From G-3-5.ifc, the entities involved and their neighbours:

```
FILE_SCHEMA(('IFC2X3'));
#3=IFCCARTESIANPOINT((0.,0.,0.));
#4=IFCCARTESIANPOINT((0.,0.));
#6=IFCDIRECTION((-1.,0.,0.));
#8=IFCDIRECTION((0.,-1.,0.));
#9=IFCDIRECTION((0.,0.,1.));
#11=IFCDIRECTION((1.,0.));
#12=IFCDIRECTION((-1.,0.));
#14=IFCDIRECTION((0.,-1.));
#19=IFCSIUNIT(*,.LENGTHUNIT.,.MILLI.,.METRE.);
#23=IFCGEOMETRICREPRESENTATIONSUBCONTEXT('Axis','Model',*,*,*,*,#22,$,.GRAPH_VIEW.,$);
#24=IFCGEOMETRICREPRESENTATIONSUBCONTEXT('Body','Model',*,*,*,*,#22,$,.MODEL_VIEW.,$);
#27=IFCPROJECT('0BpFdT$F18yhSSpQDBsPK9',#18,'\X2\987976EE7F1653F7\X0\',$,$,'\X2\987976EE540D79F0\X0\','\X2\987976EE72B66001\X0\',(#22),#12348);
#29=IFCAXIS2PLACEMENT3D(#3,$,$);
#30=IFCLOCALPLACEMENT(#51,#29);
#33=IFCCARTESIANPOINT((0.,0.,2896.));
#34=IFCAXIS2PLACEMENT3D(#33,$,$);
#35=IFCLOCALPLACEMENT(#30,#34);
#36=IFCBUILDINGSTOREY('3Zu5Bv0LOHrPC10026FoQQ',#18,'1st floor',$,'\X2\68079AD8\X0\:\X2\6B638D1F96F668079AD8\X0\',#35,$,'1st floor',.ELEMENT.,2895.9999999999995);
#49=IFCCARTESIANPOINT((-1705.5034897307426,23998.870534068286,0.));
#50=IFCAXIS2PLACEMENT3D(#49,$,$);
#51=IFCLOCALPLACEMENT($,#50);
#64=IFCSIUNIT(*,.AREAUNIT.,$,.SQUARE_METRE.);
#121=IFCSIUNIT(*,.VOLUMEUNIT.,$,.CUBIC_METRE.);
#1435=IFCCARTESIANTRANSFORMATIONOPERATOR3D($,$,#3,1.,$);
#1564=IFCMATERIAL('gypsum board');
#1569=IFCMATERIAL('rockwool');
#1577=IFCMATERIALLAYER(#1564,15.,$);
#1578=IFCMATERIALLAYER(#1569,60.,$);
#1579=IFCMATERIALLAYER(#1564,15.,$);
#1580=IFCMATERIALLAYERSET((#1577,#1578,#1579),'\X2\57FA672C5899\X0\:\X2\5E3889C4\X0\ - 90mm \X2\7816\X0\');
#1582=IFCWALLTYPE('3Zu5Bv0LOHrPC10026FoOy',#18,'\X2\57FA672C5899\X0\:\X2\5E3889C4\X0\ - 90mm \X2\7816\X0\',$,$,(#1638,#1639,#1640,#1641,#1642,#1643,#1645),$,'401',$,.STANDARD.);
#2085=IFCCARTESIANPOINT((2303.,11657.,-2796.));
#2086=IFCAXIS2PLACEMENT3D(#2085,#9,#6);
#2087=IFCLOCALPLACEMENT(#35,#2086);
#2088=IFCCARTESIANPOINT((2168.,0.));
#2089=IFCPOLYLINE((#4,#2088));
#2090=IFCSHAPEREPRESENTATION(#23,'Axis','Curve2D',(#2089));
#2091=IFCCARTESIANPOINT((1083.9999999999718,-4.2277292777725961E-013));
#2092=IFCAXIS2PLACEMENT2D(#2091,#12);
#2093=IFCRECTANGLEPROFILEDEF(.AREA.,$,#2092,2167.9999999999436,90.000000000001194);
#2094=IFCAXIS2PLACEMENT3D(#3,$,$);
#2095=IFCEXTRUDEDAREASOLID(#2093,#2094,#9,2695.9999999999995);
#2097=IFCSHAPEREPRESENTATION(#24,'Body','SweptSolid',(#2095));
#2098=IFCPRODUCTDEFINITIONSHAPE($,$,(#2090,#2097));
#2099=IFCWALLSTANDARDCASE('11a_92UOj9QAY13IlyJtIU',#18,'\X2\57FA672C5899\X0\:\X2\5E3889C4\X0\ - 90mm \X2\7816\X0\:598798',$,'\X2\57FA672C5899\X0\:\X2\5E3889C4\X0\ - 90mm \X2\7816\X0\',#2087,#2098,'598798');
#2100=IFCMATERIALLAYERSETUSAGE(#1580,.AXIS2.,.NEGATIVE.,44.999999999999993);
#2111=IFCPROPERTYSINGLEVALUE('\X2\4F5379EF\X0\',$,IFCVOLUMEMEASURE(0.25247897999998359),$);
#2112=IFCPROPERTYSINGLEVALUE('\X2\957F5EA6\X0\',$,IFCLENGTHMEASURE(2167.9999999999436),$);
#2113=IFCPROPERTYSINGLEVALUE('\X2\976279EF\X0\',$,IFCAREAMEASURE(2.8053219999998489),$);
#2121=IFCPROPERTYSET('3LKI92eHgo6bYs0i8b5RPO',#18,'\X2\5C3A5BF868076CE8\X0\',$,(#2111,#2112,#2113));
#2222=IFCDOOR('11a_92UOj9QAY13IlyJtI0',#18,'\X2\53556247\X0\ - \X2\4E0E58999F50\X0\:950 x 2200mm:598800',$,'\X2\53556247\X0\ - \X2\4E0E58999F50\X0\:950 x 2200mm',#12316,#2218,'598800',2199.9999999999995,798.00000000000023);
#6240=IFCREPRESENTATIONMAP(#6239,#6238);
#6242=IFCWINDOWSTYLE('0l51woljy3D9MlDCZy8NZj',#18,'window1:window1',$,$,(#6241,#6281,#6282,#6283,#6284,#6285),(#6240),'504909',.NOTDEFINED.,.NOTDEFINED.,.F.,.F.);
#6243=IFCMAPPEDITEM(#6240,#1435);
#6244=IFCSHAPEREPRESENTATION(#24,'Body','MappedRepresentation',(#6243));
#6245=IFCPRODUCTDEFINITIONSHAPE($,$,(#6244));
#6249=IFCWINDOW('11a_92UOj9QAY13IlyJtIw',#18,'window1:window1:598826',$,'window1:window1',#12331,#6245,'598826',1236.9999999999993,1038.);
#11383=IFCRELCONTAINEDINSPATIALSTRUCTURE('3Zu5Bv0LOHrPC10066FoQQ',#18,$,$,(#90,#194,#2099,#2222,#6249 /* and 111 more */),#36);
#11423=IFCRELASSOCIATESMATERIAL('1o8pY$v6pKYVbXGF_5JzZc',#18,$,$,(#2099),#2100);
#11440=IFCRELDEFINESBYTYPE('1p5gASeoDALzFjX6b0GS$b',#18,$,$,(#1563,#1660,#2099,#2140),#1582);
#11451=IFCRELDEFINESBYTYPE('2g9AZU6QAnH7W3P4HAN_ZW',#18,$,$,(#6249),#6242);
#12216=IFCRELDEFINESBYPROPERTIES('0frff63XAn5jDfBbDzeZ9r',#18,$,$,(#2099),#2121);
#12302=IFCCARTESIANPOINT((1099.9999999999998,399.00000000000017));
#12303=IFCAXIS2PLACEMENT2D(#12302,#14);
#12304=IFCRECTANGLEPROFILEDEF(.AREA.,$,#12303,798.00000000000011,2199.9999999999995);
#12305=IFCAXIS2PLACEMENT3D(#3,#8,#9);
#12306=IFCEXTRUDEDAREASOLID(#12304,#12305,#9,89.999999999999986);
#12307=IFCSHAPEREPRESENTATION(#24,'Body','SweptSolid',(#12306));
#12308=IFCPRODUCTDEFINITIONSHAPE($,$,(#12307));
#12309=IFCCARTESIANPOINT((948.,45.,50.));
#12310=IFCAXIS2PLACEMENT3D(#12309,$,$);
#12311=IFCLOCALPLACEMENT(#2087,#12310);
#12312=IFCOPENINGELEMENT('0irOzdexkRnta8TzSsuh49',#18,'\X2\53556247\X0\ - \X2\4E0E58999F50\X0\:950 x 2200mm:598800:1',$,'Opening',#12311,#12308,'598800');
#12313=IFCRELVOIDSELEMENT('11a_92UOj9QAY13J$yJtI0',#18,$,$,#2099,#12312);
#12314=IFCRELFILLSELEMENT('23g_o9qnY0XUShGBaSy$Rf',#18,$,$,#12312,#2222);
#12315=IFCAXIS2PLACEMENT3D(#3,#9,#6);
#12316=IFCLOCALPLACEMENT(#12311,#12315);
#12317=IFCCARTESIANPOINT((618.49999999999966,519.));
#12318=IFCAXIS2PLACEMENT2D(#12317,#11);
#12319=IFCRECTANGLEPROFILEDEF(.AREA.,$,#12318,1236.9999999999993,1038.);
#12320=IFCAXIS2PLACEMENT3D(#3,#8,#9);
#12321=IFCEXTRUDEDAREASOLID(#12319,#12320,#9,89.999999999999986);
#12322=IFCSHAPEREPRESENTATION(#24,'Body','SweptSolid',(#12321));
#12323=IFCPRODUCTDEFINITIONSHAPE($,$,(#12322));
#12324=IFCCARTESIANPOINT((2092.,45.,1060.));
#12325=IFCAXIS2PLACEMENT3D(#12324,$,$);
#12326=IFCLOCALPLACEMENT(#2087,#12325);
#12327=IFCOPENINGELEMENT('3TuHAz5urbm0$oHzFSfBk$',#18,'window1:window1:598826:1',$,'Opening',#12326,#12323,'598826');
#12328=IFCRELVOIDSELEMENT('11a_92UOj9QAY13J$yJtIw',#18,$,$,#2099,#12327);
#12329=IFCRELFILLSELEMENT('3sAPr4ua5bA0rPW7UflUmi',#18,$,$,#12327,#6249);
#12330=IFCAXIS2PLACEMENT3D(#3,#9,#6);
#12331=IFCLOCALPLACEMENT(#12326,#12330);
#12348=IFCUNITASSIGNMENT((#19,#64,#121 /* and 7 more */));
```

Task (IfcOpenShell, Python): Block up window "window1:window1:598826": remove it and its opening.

```python
import ifcopenshell
import ifcopenshell.api.feature
import ifcopenshell.api.pset
import ifcopenshell.api.root
import ifcopenshell.geom
import ifcopenshell.util.element
import ifcopenshell.util.shape
import ifcopenshell.util.unit

model = ifcopenshell.open("G-3-5.ifc")
area_scale = ifcopenshell.util.unit.calculate_unit_scale(model, "AREAUNIT")
volume_scale = ifcopenshell.util.unit.calculate_unit_scale(model, "VOLUMEUNIT")
settings = ifcopenshell.geom.settings()


def volume(element):
    """Net volume in cubic metres, openings subtracted."""
    shape = ifcopenshell.geom.create_shape(settings, element)
    return ifcopenshell.util.shape.get_volume(shape.geometry)


window = model.by_guid("11a_92UOj9QAY13IlyJtIw")
opening = window.FillsVoids[0].RelatingOpeningElement
wall = opening.VoidsElements[0].RelatingBuildingElement
before = volume(wall)

ifcopenshell.api.root.remove_product(model, product=window)
ifcopenshell.api.feature.remove_feature(model, feature=opening)

after = volume(wall)
thickness = 0.09  # wall thickness in metres

# Update the wall's stored quantities.
pset = model.by_id(ifcopenshell.util.element.get_pset(wall, "尺寸标注", should_inherit=False)["id"])
ifcopenshell.api.pset.edit_pset(model, pset=pset, properties={
    "体积": model.create_entity("IfcVolumeMeasure", after / volume_scale),
    "面积": model.create_entity("IfcAreaMeasure", after / thickness / area_scale),
})

print(f"wall volume {before:.3f} -> {after:.3f} m3")

model.write("G-3-5-out.ifc")
```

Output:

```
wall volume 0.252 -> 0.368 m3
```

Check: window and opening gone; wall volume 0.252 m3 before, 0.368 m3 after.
